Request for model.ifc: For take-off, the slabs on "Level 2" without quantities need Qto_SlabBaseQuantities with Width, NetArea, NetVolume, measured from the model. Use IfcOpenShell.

First a look at what the model holds.

```python
import ifcopenshell
import ifcopenshell.util.element
import ifcopenshell.util.unit

model = ifcopenshell.open("model.ifc")
print(model.schema)
for unit_type in ("LENGTHUNIT", "AREAUNIT", "VOLUMEUNIT"):
    print(unit_type, ifcopenshell.util.unit.calculate_unit_scale(model, unit_type))
storey = next(s for s in model.by_type("IfcBuildingStorey") if s.Name == "Level 2")
slabs = [e for e in ifcopenshell.util.element.get_decomposition(storey) if e.is_a("IfcSlab")]
for e in sorted(slabs, key=lambda e: e.id()):
    print(e.id(), e.is_a(), e.Name, list(ifcopenshell.util.element.get_psets(e, qtos_only=True)), sep=" | ")
```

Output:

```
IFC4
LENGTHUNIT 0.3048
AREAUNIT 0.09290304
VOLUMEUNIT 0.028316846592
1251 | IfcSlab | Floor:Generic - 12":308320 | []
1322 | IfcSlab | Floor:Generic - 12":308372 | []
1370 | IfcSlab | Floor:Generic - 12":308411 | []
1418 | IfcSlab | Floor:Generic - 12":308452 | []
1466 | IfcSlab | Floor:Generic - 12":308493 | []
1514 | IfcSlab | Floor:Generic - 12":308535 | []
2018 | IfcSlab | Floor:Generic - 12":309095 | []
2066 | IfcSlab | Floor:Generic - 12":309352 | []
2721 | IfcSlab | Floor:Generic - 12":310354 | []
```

```python
import ifcopenshell
import ifcopenshell.api.pset
import ifcopenshell.geom
import ifcopenshell.util.element
import ifcopenshell.util.shape
import ifcopenshell.util.unit

model = ifcopenshell.open("model.ifc")
unit_scale = ifcopenshell.util.unit.calculate_unit_scale(model)
area_scale = ifcopenshell.util.unit.calculate_unit_scale(model, "AREAUNIT")
volume_scale = ifcopenshell.util.unit.calculate_unit_scale(model, "VOLUMEUNIT")
settings = ifcopenshell.geom.settings()

storey = next(s for s in model.by_type("IfcBuildingStorey") if s.Name == "Level 2")
slabs = [e for e in ifcopenshell.util.element.get_decomposition(storey) if e.is_a("IfcSlab")]

for e in sorted(slabs, key=lambda e: e.id()):
    if ifcopenshell.util.element.get_psets(e, qtos_only=True, should_inherit=False):
        continue
    # Geometry comes back in metres, in the element's own axes.
    shape = ifcopenshell.geom.create_shape(settings, e)
    values = {
        "Width": ifcopenshell.util.shape.get_z(shape.geometry) / unit_scale,
        "NetArea": ifcopenshell.util.shape.get_footprint_area(shape.geometry) / area_scale,
        "NetVolume": ifcopenshell.util.shape.get_volume(shape.geometry) / volume_scale,
    }
    qto = ifcopenshell.api.pset.add_qto(model, product=e, name="Qto_SlabBaseQuantities")
    ifcopenshell.api.pset.edit_qto(model, qto=qto, properties=values)
    print(e.id(), {k: round(v, 3) for k, v in values.items()})

model.write("model_rev.ifc")
```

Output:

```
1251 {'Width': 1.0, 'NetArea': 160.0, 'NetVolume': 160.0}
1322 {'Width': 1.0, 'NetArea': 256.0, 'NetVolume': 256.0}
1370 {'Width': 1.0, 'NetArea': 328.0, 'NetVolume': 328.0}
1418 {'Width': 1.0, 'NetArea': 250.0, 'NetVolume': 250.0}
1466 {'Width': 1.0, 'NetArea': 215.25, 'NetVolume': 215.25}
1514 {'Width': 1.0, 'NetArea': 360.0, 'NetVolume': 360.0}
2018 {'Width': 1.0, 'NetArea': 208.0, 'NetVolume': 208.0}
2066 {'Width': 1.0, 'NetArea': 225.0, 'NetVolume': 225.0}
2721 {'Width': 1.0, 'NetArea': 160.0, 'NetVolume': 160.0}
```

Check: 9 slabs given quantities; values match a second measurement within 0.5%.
